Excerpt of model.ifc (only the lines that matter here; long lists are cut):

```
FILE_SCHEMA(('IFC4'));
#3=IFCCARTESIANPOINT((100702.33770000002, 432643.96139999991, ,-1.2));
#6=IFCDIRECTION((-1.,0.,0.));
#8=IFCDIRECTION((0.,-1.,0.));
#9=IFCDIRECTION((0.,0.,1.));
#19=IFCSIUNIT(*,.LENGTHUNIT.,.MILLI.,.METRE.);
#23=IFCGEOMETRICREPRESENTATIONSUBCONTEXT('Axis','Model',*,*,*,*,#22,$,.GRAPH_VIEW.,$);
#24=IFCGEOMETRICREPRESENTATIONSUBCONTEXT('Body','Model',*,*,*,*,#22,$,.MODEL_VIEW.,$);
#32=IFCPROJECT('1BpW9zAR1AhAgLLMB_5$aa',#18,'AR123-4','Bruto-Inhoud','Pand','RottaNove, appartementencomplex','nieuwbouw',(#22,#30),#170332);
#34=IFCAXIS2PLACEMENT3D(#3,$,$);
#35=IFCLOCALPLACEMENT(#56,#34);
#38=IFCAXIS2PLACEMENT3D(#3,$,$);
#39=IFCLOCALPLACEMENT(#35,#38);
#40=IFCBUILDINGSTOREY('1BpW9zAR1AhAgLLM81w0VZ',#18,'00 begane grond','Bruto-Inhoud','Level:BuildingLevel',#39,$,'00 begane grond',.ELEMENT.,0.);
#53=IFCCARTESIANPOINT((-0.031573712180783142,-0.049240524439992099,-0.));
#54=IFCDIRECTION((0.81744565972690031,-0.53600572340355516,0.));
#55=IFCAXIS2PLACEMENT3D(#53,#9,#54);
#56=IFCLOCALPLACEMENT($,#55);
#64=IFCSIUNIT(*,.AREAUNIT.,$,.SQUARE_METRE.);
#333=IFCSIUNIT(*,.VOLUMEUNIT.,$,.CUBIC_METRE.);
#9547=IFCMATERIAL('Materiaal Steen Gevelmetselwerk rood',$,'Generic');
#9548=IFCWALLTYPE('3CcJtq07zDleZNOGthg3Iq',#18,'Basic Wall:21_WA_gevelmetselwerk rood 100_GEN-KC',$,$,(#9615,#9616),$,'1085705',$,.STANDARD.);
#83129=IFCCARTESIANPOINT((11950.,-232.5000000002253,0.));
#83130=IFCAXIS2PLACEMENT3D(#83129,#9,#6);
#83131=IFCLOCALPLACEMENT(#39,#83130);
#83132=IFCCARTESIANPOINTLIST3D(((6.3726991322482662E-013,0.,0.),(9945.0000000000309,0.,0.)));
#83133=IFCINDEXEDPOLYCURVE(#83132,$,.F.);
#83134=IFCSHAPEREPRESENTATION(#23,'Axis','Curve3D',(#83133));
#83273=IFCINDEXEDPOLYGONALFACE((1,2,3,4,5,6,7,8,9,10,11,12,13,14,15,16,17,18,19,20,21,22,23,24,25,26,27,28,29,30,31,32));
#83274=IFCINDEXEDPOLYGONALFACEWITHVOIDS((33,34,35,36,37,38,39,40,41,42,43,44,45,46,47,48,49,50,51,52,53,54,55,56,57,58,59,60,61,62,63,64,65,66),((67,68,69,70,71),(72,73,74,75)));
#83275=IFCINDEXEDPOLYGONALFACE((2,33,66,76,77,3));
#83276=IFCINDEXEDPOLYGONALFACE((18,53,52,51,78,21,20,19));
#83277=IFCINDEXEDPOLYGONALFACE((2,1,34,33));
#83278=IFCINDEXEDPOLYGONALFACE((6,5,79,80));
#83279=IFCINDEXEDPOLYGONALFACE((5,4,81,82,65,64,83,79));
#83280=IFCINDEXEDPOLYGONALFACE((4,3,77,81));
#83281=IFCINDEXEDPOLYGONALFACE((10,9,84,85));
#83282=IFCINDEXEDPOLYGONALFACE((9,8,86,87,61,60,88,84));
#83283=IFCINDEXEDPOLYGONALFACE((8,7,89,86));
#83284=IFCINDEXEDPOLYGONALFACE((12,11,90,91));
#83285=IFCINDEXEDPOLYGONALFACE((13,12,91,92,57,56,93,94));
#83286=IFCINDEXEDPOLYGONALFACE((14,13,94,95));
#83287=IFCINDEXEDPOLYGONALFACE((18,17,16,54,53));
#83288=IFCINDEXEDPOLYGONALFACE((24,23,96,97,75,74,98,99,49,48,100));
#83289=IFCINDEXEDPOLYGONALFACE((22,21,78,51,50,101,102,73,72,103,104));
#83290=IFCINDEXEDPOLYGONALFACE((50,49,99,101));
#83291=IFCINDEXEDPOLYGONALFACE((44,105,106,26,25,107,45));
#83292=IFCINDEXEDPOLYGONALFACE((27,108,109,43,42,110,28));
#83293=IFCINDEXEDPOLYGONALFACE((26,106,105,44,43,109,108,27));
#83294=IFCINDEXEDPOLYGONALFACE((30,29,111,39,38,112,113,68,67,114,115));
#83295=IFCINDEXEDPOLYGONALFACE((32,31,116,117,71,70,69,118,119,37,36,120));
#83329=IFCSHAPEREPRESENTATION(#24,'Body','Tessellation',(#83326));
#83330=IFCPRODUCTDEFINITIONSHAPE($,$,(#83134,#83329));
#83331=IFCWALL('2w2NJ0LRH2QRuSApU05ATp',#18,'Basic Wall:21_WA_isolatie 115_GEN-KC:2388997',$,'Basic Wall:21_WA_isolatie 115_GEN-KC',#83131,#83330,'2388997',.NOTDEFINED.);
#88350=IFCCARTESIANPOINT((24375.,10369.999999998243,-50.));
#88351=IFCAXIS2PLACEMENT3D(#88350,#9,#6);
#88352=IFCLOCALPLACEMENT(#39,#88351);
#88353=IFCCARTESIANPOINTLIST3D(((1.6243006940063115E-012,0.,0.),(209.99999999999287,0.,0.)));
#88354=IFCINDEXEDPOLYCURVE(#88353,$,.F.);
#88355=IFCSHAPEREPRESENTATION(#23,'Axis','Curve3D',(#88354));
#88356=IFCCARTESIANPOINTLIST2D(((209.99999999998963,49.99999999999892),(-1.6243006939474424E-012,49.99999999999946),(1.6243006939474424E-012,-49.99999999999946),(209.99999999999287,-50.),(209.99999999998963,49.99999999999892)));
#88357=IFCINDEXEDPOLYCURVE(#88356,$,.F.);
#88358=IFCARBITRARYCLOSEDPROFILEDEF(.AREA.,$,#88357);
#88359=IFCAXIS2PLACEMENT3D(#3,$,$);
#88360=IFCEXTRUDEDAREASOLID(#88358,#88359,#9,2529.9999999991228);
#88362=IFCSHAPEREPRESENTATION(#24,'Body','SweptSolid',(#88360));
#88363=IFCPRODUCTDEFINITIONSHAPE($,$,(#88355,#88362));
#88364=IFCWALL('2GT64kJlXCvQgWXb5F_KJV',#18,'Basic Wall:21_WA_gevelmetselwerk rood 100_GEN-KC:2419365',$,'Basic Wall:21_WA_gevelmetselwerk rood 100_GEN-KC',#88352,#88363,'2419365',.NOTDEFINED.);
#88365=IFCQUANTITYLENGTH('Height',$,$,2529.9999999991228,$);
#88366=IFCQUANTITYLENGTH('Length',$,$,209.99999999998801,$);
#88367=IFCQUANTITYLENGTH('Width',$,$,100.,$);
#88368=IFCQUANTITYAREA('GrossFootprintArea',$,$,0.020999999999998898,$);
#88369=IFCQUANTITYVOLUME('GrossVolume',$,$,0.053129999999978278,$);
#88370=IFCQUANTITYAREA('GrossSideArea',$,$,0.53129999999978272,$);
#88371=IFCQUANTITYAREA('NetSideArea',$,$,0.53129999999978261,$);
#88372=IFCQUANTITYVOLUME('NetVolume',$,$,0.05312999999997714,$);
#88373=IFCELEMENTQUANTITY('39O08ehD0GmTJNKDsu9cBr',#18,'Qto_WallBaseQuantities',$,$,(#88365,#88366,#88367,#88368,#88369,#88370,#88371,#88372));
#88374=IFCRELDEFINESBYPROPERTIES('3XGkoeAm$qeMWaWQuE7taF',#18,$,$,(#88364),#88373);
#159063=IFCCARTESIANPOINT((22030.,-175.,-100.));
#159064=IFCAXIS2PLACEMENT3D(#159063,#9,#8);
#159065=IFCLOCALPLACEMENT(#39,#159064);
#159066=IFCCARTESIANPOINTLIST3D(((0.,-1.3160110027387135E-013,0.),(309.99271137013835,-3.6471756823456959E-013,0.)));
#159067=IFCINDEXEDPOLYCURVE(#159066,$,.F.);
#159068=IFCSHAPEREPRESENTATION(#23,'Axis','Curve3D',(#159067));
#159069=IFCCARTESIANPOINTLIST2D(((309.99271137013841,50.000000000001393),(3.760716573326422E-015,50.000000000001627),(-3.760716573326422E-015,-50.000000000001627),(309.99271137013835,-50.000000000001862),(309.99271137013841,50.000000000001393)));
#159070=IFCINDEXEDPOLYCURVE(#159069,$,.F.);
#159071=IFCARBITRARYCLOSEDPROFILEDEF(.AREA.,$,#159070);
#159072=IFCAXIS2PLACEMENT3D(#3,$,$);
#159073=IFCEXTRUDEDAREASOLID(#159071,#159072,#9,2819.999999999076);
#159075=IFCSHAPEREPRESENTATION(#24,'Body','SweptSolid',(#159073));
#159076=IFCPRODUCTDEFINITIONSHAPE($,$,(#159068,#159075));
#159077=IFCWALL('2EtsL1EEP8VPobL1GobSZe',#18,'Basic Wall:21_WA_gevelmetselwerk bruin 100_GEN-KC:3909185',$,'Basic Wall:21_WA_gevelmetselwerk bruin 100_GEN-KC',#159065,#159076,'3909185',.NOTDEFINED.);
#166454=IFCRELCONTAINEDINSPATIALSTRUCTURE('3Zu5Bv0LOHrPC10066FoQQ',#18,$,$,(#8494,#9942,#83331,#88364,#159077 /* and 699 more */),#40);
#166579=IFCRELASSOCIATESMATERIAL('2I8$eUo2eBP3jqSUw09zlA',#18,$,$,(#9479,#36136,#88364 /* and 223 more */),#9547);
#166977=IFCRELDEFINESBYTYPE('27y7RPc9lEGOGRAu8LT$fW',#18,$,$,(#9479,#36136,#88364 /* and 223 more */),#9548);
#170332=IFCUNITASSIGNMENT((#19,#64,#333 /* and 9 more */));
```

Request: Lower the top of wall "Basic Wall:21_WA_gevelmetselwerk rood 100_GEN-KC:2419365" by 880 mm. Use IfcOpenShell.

```python
import ifcopenshell
import ifcopenshell.api.pset
import ifcopenshell.geom
import ifcopenshell.util.element
import ifcopenshell.util.representation
import ifcopenshell.util.shape
import ifcopenshell.util.unit

model = ifcopenshell.open("model.ifc")
unit_scale = ifcopenshell.util.unit.calculate_unit_scale(model)
area_scale = ifcopenshell.util.unit.calculate_unit_scale(model, "AREAUNIT")
volume_scale = ifcopenshell.util.unit.calculate_unit_scale(model, "VOLUMEUNIT")
settings = ifcopenshell.geom.settings()


def volume(element):
    """Net volume in cubic metres, openings subtracted."""
    shape = ifcopenshell.geom.create_shape(settings, element)
    return ifcopenshell.util.shape.get_volume(shape.geometry)


wall = model.by_guid("2GT64kJlXCvQgWXb5F_KJV")
before = volume(wall)

body = ifcopenshell.util.representation.get_representation(wall, "Model", "Body")
solid = body.Items[0]
old_height = solid.Depth
solid.Depth -= 0.88 / unit_scale
after = volume(wall)
thickness = 0.1  # wall thickness in metres

# Update the stored height, areas and volumes.
qto = model.by_id(ifcopenshell.util.element.get_pset(wall, "Qto_WallBaseQuantities", should_inherit=False)["id"])
ifcopenshell.api.pset.edit_qto(model, qto=qto, properties={
    "Height": solid.Depth,
    "GrossVolume": ifcopenshell.util.element.get_pset(wall, "Qto_WallBaseQuantities", "GrossVolume") * solid.Depth / old_height,
    "GrossSideArea": ifcopenshell.util.element.get_pset(wall, "Qto_WallBaseQuantities", "GrossSideArea") * solid.Depth / old_height,
    "NetSideArea": after / thickness / area_scale,
    "NetVolume": after / volume_scale,
})

print(f"height {old_height:g} -> {solid.Depth:g}, volume {before:.3f} -> {after:.3f} m3")

model.write("model-out.ifc")
```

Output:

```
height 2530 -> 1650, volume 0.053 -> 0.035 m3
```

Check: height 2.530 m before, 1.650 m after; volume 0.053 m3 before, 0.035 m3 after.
